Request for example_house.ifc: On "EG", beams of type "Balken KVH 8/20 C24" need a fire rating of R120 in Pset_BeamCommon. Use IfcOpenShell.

First a look at what the model holds.

```python
import ifcopenshell
import ifcopenshell.util.element

model = ifcopenshell.open("example_house.ifc")
print(model.schema)
storey = next(s for s in model.by_type("IfcBuildingStorey") if s.Name == "EG")
beams = [e for e in ifcopenshell.util.element.get_decomposition(storey) if e.is_a("IfcBeam")]
seen = {}
for e in beams:
    element_type = ifcopenshell.util.element.get_type(e)
    key = (element_type.Name if element_type != e and element_type else None, ifcopenshell.util.element.get_pset(e, "Pset_BeamCommon", "FireRating"))
    seen[key] = seen.get(key, 0) + 1
for (name, value), count in sorted(seen.items(), key=str):
    print(count, "x", name, "|", value)
```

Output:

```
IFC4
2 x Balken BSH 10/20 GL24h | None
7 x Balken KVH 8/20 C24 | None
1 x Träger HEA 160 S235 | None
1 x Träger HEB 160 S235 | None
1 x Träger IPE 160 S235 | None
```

```python
import ifcopenshell
import ifcopenshell.api.pset
import ifcopenshell.util.element

model = ifcopenshell.open("example_house.ifc")

storey = next(s for s in model.by_type("IfcBuildingStorey") if s.Name == "EG")
beams = [e for e in ifcopenshell.util.element.get_decomposition(storey) if e.is_a("IfcBeam")]

count = 0
for e in beams:
    element_type = ifcopenshell.util.element.get_type(e)
    if element_type in (None, e) or element_type.Name != "Balken KVH 8/20 C24":
        continue
    # add_pset returns the element's existing set when there is one.
    pset = ifcopenshell.api.pset.add_pset(model, product=e, name="Pset_BeamCommon")
    ifcopenshell.api.pset.edit_pset(model, pset=pset, properties={"FireRating": "R120"})
    count += 1

print(count, "beams updated")

model.write("example_house_rev.ifc")
```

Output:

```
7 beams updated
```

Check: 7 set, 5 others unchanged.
